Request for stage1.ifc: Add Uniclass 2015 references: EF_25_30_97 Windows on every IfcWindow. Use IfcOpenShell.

First a look at what the model holds.

```python
import ifcopenshell

model = ifcopenshell.open("stage1.ifc")
print(model.schema)
print("classifications:", [c.Name for c in model.by_type("IfcClassification")])
for ifc_class in ("IfcDoor", "IfcRoof", "IfcStair", "IfcWall", "IfcWindow"):
    print(ifc_class, len(model.by_type(ifc_class)))
```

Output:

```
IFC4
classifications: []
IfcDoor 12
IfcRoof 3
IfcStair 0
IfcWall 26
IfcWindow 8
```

```python
import ifcopenshell
import ifcopenshell.api.classification

model = ifcopenshell.open("stage1.ifc")

system = ifcopenshell.api.classification.add_classification(model, classification="Uniclass 2015")

codes = {
    "IfcWindow": ("EF_25_30_97", "Windows"),
}
for ifc_class, (code, name) in codes.items():
    products = model.by_type(ifc_class)
    ifcopenshell.api.classification.add_reference(
        model, products=products, classification=system, identification=code, name=name
    )
    print(code, len(products))

model.write("stage1_v2.ifc")
```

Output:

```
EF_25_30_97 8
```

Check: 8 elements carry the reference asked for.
